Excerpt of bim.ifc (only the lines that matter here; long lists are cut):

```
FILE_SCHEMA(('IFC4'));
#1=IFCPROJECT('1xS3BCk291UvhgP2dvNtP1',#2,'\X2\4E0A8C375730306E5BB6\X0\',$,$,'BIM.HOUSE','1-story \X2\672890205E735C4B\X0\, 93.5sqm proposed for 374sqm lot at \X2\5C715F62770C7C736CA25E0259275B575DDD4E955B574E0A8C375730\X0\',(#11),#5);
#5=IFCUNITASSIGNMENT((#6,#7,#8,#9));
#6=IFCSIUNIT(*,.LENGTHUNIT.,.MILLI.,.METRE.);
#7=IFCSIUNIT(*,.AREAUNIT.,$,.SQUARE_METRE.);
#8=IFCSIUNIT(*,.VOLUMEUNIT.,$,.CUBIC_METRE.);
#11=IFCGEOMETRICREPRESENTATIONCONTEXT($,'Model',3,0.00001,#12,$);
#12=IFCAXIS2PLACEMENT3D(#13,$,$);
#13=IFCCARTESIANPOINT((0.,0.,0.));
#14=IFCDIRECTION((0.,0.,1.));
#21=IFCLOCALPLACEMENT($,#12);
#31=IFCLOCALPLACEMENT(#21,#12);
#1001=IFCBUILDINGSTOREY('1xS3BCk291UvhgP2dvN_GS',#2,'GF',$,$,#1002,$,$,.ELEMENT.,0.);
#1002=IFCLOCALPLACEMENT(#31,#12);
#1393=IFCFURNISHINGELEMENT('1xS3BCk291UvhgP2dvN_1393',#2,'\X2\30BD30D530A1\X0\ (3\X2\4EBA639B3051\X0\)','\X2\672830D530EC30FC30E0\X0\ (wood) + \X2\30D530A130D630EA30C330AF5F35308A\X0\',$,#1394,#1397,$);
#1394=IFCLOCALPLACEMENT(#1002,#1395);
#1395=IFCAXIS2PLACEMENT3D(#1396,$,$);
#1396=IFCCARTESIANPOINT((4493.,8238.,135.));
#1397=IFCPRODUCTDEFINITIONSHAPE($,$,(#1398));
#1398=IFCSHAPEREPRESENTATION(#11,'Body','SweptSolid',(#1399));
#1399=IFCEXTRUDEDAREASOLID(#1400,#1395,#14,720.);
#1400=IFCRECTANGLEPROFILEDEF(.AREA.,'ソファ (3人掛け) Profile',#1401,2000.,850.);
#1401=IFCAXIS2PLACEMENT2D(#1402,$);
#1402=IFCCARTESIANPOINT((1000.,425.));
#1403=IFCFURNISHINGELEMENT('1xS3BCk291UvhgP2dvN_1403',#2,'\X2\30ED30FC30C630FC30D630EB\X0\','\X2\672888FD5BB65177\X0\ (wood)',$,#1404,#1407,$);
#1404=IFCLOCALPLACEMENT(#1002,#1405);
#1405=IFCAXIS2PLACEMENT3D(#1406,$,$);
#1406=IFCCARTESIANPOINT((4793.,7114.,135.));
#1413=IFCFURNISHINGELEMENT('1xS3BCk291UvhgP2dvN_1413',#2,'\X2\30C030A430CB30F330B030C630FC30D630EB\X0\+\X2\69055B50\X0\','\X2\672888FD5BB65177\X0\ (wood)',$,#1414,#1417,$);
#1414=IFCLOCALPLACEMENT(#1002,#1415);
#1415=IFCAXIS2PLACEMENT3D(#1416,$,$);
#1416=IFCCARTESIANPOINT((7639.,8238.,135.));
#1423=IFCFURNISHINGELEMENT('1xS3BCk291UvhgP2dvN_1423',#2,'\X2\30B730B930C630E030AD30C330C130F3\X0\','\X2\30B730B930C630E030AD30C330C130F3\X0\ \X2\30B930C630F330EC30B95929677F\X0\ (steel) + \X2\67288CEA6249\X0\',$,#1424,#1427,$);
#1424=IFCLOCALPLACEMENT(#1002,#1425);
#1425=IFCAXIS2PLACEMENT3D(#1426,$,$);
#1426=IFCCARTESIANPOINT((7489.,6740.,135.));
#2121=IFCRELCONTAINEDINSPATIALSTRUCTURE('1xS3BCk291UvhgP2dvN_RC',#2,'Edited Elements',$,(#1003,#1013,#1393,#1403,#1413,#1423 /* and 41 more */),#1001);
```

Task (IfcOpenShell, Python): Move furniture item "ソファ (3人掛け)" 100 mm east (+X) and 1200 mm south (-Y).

```python
import ifcopenshell
import ifcopenshell.api.geometry
import ifcopenshell.util.placement

model = ifcopenshell.open("bim.ifc")

item = model.by_guid("1xS3BCk291UvhgP2dvN_1393")
matrix = ifcopenshell.util.placement.get_local_placement(item.ObjectPlacement)
matrix[0, 3] += 100.0
matrix[1, 3] -= 1200.0
ifcopenshell.api.geometry.edit_object_placement(model, product=item, matrix=matrix, is_si=False)

print(ifcopenshell.util.placement.get_local_placement(item.ObjectPlacement).round(3) + 0.0)

model.write("bim-out.ifc")
```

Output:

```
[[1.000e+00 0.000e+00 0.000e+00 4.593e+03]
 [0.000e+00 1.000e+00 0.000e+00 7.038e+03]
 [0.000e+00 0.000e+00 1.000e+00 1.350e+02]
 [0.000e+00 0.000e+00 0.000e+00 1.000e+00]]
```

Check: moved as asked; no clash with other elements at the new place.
